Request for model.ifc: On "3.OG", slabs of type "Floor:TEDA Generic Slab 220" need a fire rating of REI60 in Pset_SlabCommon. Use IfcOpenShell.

First a look at what the model holds.

```python
import ifcopenshell
import ifcopenshell.util.element

model = ifcopenshell.open("model.ifc")
print(model.schema)
storey = next(s for s in model.by_type("IfcBuildingStorey") if s.Name == "3.OG")
slabs = [e for e in ifcopenshell.util.element.get_decomposition(storey) if e.is_a("IfcSlab")]
seen = {}
for e in slabs:
    element_type = ifcopenshell.util.element.get_type(e)
    key = (element_type.Name if element_type != e and element_type else None, ifcopenshell.util.element.get_pset(e, "Pset_SlabCommon", "FireRating"))
    seen[key] = seen.get(key, 0) + 1
for (name, value), count in sorted(seen.items(), key=str):
    print(count, "x", name, "|", value)
```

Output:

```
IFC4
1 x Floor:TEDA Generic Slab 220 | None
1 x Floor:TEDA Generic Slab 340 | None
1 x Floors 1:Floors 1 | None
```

```python
import ifcopenshell
import ifcopenshell.api.pset
import ifcopenshell.util.element

model = ifcopenshell.open("model.ifc")

storey = next(s for s in model.by_type("IfcBuildingStorey") if s.Name == "3.OG")
slabs = [e for e in ifcopenshell.util.element.get_decomposition(storey) if e.is_a("IfcSlab")]

count = 0
for e in slabs:
    element_type = ifcopenshell.util.element.get_type(e)
    if element_type in (None, e) or element_type.Name != "Floor:TEDA Generic Slab 220":
        continue
    # add_pset returns the element's existing set when there is one.
    pset = ifcopenshell.api.pset.add_pset(model, product=e, name="Pset_SlabCommon")
    ifcopenshell.api.pset.edit_pset(model, pset=pset, properties={"FireRating": "REI60"})
    count += 1

print(count, "slabs updated")

model.write("model_v2.ifc")
```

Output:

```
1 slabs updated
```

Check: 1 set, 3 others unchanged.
